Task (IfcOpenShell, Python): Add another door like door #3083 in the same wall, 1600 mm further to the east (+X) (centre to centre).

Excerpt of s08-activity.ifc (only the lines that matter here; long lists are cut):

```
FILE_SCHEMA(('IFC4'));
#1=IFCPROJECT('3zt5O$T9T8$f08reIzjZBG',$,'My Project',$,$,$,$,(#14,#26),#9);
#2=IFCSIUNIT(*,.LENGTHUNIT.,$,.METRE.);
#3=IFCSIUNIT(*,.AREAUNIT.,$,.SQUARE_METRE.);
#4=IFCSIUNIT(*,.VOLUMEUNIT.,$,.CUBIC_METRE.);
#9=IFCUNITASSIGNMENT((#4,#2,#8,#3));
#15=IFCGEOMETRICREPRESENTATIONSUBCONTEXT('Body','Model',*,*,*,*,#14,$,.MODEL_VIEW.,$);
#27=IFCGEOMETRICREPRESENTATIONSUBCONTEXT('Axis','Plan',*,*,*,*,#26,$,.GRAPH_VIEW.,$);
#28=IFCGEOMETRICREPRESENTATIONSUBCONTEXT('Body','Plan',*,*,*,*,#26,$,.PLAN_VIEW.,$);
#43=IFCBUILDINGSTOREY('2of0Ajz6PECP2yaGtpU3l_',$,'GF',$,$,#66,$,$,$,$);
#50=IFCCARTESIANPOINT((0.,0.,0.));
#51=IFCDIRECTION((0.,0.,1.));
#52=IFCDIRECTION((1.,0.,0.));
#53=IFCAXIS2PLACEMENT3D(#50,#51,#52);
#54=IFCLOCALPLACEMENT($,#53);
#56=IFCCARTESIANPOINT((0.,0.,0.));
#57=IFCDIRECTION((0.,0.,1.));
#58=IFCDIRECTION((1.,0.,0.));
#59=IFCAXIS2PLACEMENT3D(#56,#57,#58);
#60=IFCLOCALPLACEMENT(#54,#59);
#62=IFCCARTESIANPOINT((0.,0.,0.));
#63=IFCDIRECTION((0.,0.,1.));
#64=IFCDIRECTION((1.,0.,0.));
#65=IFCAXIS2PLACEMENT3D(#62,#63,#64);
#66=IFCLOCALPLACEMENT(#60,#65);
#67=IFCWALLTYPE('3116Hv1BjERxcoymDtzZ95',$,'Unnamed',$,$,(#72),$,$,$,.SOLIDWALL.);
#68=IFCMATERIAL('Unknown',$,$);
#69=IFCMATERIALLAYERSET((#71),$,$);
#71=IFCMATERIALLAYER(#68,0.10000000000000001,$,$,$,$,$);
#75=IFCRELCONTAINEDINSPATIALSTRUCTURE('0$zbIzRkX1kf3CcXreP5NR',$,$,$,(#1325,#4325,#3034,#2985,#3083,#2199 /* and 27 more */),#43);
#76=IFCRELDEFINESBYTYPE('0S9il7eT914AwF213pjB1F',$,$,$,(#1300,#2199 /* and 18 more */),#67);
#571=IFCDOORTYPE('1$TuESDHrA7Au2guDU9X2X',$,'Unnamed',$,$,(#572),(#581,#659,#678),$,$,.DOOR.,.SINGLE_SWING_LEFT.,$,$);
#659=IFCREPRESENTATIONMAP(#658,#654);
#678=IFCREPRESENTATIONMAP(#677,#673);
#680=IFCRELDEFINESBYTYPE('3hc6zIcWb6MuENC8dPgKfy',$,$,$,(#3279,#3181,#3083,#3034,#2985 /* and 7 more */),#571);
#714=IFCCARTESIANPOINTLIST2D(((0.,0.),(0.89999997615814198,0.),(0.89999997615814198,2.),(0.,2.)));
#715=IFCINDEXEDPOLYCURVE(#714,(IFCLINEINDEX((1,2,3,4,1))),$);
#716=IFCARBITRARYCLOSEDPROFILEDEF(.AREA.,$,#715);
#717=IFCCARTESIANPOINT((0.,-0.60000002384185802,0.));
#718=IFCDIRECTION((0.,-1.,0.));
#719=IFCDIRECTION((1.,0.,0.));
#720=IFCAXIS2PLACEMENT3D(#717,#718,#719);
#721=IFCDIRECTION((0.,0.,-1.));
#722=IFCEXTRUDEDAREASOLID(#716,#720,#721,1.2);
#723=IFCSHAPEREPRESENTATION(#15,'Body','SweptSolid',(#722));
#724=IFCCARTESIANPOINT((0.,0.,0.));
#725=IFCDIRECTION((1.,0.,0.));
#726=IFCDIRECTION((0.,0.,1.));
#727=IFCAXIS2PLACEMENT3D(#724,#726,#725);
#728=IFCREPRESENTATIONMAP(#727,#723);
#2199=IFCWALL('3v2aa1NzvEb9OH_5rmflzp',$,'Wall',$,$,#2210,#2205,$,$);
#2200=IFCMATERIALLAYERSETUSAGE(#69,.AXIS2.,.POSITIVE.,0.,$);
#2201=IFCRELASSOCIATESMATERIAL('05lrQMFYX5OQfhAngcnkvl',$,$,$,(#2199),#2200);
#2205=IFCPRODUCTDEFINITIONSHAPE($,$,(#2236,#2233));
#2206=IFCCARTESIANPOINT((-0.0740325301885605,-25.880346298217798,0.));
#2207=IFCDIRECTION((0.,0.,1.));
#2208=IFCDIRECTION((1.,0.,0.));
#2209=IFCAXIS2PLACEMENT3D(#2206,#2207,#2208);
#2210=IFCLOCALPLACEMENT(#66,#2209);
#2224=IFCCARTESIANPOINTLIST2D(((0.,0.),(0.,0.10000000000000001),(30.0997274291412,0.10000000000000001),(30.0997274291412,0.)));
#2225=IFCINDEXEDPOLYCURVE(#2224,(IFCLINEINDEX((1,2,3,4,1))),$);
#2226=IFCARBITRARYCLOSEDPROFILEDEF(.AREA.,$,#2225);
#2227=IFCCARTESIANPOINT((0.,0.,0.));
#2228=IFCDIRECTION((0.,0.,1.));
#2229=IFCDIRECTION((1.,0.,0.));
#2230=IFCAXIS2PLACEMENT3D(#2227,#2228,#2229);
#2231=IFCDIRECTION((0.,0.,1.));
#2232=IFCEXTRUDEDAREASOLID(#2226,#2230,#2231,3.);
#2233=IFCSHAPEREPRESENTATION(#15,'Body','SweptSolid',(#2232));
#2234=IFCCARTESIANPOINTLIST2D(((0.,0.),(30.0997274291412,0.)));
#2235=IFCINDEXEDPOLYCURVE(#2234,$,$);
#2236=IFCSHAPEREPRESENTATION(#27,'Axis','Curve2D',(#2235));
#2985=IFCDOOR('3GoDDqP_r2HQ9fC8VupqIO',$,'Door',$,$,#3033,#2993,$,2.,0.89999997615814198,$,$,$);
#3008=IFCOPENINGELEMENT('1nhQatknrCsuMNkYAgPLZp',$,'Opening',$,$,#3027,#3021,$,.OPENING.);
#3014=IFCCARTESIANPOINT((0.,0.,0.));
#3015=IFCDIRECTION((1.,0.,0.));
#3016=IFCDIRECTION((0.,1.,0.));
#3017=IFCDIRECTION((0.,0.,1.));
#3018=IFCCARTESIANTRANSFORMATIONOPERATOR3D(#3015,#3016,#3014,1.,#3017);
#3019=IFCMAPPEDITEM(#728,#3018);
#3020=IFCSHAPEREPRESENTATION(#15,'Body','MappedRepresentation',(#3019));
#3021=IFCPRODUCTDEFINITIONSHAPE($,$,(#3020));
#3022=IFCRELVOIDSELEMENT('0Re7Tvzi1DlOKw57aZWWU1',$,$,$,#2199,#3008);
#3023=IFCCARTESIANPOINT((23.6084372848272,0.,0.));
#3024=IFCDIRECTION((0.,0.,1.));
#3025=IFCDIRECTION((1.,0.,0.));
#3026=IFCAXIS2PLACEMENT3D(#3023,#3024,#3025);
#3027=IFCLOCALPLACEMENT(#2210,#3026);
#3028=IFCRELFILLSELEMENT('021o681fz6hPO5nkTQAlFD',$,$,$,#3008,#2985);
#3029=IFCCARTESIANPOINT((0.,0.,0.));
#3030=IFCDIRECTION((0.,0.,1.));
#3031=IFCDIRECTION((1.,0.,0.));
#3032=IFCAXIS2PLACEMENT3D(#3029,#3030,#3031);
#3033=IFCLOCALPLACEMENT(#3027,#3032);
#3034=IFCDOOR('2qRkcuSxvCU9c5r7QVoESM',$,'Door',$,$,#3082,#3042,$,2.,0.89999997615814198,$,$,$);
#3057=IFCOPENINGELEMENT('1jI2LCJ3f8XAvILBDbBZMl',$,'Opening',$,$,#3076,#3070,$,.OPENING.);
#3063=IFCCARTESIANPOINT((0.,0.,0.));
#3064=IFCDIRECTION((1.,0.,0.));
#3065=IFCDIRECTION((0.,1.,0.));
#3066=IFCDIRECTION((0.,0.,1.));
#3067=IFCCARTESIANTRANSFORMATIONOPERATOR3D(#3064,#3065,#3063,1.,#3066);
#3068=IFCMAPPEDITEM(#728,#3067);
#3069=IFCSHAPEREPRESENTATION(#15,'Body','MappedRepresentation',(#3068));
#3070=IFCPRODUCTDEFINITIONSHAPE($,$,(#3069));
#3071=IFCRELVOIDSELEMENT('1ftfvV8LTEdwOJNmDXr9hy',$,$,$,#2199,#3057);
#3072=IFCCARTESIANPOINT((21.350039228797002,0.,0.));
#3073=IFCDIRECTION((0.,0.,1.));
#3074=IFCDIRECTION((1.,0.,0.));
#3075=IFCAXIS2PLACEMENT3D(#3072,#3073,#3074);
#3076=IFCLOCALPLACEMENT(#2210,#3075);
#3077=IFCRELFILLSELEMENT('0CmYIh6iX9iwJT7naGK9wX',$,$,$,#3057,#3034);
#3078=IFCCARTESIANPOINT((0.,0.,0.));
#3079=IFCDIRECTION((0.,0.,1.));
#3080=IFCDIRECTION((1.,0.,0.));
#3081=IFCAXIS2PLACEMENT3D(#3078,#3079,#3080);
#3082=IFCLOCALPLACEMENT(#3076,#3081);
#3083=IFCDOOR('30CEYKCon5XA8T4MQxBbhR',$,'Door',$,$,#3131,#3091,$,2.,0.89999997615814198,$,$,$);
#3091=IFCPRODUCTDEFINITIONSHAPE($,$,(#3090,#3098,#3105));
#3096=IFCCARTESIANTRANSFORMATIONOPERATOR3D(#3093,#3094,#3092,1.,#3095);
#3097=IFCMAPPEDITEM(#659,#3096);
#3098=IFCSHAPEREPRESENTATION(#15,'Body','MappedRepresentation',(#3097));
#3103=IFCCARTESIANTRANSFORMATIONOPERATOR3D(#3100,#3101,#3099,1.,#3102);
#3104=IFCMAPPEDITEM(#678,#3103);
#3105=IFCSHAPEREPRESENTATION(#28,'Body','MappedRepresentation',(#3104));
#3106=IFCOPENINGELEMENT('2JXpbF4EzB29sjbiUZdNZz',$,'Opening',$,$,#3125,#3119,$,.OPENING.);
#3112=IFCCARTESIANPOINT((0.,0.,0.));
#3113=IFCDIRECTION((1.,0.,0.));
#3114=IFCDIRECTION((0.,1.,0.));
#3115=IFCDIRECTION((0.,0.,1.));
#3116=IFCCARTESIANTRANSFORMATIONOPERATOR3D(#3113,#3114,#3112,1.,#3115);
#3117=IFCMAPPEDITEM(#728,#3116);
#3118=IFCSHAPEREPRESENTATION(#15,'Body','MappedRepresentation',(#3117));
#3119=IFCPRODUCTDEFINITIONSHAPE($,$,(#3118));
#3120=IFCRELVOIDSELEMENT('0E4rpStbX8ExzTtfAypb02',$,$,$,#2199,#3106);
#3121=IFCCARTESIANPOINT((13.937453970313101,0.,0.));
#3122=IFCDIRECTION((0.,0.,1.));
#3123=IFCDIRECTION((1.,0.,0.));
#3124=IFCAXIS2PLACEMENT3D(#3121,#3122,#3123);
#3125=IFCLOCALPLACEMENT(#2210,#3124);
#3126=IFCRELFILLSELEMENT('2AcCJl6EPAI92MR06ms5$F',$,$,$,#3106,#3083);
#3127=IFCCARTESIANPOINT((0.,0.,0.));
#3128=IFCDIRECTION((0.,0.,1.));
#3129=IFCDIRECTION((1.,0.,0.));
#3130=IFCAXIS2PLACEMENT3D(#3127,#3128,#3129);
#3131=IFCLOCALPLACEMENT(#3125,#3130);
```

```python
import ifcopenshell
import ifcopenshell.api.feature
import ifcopenshell.api.geometry
import ifcopenshell.api.root
import ifcopenshell.geom
import ifcopenshell.util.element
import ifcopenshell.util.placement
import ifcopenshell.util.shape

model = ifcopenshell.open("s08-activity.ifc")
settings = ifcopenshell.geom.settings()


def volume(element):
    """Net volume in cubic metres, openings subtracted."""
    shape = ifcopenshell.geom.create_shape(settings, element)
    return ifcopenshell.util.shape.get_volume(shape.geometry)


door = model.by_guid("30CEYKCon5XA8T4MQxBbhR")
opening = door.FillsVoids[0].RelatingOpeningElement
wall = opening.VoidsElements[0].RelatingBuildingElement
before = volume(wall)
shift = ifcopenshell.util.placement.get_local_placement(wall.ObjectPlacement)[:3, 0] * 1.6

# copy_class copies the void relationship, type, container and properties, but no geometry.
new_opening = ifcopenshell.api.root.copy_class(model, product=opening)
new_opening.Representation = ifcopenshell.util.element.copy_deep(
    model, opening.Representation, exclude=["IfcGeometricRepresentationContext", "IfcRepresentationMap"]
)
new_door = ifcopenshell.api.root.copy_class(model, product=door)
new_door.Representation = ifcopenshell.util.element.copy_deep(
    model, door.Representation, exclude=["IfcGeometricRepresentationContext", "IfcRepresentationMap"]
)
ifcopenshell.api.feature.add_filling(model, opening=new_opening, element=new_door)

for old, new in ((opening, new_opening), (door, new_door)):
    matrix = ifcopenshell.util.placement.get_local_placement(old.ObjectPlacement)
    matrix[:3, 3] += shift
    ifcopenshell.api.geometry.edit_object_placement(model, product=new, matrix=matrix, is_si=False)

after = volume(wall)

print(f"wall volume {before:.3f} -> {after:.3f} m3")

model.write("s08-activity_updated.ifc")
```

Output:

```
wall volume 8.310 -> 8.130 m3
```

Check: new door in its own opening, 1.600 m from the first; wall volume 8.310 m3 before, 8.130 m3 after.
